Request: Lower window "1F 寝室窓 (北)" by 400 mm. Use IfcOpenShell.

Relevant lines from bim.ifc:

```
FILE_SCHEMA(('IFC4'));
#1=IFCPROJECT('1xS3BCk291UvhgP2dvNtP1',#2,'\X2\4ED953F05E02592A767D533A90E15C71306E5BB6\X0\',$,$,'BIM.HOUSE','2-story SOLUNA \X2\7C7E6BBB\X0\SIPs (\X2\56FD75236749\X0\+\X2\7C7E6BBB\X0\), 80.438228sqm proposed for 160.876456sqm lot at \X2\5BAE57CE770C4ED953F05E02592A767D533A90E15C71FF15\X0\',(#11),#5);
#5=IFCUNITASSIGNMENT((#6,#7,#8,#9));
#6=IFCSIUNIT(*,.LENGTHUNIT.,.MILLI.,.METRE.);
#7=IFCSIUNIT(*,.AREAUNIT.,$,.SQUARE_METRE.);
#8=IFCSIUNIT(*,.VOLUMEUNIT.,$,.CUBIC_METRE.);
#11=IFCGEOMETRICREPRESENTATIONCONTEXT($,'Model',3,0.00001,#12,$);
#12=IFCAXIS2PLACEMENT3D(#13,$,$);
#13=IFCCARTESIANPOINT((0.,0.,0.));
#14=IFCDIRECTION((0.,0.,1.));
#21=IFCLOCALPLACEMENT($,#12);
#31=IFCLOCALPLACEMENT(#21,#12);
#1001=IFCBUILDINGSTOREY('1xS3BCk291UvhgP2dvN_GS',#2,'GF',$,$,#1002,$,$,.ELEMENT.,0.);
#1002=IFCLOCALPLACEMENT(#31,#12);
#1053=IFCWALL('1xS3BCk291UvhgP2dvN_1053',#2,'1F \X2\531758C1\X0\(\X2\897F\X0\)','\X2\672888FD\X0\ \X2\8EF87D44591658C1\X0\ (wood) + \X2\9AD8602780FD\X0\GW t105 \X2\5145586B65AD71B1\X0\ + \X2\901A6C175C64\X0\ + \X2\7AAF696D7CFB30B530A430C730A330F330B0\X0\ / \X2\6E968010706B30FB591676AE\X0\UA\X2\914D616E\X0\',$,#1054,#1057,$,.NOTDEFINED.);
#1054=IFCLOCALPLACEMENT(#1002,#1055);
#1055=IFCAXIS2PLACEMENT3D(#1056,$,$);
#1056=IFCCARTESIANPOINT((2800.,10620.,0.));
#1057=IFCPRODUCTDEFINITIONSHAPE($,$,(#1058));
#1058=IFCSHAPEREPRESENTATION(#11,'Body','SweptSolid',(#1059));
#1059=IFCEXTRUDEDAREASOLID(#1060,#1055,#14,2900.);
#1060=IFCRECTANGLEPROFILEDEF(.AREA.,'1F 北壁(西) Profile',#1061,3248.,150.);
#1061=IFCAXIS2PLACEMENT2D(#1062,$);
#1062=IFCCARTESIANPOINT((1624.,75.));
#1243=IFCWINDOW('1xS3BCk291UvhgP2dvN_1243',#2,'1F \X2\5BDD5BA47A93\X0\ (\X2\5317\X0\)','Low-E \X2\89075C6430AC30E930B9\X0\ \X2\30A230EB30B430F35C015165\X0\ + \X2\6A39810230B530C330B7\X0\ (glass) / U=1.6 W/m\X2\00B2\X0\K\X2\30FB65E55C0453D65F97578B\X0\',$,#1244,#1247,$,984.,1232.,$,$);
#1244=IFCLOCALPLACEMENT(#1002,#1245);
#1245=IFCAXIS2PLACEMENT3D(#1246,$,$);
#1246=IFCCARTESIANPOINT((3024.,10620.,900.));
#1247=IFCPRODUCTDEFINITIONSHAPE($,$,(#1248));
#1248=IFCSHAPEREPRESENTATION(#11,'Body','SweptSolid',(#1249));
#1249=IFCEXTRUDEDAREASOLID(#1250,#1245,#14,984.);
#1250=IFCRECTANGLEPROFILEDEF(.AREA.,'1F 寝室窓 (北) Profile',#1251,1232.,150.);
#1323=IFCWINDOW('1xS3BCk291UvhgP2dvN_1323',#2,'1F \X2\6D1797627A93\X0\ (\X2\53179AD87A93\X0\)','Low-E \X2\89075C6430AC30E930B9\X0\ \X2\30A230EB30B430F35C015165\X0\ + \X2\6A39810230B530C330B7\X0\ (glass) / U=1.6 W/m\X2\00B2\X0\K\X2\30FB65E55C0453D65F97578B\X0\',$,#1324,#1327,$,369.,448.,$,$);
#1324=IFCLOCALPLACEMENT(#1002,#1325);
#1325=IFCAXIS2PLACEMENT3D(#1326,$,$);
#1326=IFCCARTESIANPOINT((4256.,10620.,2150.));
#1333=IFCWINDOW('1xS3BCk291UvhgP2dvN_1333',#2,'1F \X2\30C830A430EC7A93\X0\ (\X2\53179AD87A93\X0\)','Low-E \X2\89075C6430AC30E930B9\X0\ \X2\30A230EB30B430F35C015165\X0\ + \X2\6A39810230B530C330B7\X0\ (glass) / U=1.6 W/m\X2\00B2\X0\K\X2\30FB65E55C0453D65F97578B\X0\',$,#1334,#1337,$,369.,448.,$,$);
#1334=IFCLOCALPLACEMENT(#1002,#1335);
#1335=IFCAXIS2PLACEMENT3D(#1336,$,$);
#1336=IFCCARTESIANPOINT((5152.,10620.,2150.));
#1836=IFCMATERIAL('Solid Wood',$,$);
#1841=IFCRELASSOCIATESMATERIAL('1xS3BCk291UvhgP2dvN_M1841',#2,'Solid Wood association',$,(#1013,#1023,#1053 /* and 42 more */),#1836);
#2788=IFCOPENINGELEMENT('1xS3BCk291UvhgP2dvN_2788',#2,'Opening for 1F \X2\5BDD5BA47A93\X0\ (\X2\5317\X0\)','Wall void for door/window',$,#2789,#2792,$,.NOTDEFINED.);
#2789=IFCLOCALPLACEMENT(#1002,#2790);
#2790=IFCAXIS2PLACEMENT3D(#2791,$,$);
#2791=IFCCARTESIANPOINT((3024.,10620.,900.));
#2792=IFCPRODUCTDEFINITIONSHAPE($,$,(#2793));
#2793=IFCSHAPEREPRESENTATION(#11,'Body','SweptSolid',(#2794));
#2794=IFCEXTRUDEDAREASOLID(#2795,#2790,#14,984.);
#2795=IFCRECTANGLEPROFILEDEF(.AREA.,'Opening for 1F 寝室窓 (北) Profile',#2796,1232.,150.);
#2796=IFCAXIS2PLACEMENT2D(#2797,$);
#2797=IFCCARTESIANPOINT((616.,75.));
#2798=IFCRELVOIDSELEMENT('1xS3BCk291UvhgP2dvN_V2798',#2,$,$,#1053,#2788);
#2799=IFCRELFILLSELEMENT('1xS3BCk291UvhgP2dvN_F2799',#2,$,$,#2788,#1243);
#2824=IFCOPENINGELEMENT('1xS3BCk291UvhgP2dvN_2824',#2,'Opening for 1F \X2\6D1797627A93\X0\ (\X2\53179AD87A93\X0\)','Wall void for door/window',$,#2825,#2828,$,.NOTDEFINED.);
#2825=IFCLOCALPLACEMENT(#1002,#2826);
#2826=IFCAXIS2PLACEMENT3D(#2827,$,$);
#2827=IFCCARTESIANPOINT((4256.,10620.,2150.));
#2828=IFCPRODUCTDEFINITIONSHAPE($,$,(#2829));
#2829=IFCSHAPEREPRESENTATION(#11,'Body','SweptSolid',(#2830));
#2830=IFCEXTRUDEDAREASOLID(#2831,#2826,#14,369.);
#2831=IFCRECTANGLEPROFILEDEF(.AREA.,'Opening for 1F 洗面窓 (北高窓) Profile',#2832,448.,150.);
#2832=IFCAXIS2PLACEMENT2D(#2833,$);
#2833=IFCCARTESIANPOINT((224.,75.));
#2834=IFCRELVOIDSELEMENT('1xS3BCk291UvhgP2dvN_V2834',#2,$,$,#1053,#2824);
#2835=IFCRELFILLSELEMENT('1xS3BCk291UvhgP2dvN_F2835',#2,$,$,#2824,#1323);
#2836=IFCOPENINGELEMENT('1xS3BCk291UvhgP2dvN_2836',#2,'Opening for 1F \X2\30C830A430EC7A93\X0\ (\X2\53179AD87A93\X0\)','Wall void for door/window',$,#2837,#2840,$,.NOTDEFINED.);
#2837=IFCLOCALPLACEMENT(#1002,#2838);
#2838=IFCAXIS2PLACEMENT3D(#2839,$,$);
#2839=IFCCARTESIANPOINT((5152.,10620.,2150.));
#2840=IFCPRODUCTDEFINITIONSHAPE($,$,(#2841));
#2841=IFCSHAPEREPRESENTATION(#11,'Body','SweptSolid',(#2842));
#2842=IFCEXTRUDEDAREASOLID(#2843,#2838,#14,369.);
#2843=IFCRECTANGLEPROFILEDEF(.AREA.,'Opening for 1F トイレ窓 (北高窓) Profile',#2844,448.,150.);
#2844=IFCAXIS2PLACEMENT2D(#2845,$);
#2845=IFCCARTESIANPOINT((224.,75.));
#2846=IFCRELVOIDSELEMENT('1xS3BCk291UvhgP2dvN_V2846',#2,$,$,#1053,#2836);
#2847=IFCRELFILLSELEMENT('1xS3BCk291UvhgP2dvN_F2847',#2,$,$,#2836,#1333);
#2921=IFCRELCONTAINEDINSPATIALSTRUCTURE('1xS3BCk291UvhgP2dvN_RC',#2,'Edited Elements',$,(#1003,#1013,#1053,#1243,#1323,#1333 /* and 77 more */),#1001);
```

```python
import numpy as np
import ifcopenshell
import ifcopenshell.api.geometry
import ifcopenshell.util.placement
import ifcopenshell.util.unit

model = ifcopenshell.open("bim.ifc")
unit_scale = ifcopenshell.util.unit.calculate_unit_scale(model)

window = model.by_id(1243)
opening = window.FillsVoids[0].RelatingOpeningElement
dz = -0.4 / unit_scale

shift = np.array([0.0, 0.0, dz])
# The window is not placed relative to its opening, so move both.
for product in (opening, window):
    matrix = ifcopenshell.util.placement.get_local_placement(product.ObjectPlacement)
    matrix[:3, 3] += shift
    ifcopenshell.api.geometry.edit_object_placement(model, product=product, matrix=matrix, is_si=False)

print(f"moved by {dz * unit_scale:+.3f} m")

model.write("bim_v2.ifc")
```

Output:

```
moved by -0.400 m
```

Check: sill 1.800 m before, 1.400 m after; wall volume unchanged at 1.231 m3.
